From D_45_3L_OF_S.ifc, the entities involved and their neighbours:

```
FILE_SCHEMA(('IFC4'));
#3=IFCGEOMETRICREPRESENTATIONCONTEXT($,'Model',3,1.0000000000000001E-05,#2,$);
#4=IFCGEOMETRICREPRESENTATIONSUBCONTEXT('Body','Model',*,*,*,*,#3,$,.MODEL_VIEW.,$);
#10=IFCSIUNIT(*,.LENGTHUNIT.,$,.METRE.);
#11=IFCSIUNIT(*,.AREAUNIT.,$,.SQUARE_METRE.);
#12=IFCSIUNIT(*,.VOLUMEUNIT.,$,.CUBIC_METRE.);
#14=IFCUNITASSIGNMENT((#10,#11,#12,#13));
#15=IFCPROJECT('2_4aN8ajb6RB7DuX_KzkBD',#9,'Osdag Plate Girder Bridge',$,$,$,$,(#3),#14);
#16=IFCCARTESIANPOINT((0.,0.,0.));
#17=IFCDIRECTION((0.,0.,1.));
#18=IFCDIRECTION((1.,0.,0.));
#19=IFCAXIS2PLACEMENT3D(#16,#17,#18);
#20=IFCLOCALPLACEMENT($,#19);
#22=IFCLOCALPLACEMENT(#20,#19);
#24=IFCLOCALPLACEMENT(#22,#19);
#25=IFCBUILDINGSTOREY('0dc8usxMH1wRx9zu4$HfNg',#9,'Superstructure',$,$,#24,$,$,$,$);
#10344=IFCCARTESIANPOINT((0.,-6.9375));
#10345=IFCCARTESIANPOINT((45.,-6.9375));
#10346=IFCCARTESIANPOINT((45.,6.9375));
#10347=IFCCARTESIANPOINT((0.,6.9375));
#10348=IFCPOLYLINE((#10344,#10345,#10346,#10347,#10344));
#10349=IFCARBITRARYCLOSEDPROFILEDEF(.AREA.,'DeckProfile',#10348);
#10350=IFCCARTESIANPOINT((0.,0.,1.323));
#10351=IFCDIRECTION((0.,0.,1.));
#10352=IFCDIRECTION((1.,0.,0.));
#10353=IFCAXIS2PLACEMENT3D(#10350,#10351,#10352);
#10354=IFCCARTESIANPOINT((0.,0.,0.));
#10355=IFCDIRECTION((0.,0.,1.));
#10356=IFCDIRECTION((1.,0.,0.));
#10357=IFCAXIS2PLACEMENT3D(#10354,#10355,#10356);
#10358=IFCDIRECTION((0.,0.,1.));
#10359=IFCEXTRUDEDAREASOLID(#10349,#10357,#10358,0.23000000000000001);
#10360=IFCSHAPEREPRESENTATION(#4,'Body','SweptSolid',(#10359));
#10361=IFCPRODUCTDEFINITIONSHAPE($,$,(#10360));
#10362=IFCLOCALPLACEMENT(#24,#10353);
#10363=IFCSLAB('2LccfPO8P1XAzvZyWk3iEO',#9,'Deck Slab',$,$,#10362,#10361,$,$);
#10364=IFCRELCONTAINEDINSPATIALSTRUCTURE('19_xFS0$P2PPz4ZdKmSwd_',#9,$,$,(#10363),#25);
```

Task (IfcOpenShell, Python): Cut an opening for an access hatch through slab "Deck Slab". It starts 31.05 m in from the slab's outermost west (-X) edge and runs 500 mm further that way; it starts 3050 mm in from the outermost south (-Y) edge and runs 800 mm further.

```python
import numpy as np
import ifcopenshell
import ifcopenshell.api.feature
import ifcopenshell.api.geometry
import ifcopenshell.api.root
import ifcopenshell.geom
import ifcopenshell.util.placement
import ifcopenshell.util.representation
import ifcopenshell.util.shape
import ifcopenshell.util.unit

model = ifcopenshell.open("D_45_3L_OF_S.ifc")
unit_scale = ifcopenshell.util.unit.calculate_unit_scale(model)
settings = ifcopenshell.geom.settings()


def volume(element):
    """Net volume in cubic metres, openings subtracted."""
    shape = ifcopenshell.geom.create_shape(settings, element)
    return ifcopenshell.util.shape.get_volume(shape.geometry)


slab = model.by_id(10363)
before = volume(slab)

# Extent in the slab's own axes, in metres. The edges named are its -X and -Y sides.
slab_shape = ifcopenshell.geom.create_shape(settings, slab)
vertices = ifcopenshell.util.shape.get_vertices(slab_shape.geometry)
x_min, y_min, bottom = vertices.min(axis=0)
top = vertices[:, 2].max()

opening = ifcopenshell.api.root.create_entity(model, ifc_class="IfcOpeningElement", name="Access hatch opening", predefined_type="OPENING")
context = ifcopenshell.util.representation.get_context(model, "Model", "Body", "MODEL_VIEW")
width, depth = 0.5, 0.8
outline = [(0.0, 0.0), (width, 0.0), (width, depth), (0.0, depth), (0.0, 0.0)]
# Overshoot both faces by 50 mm so the cut is clean.
shape = ifcopenshell.api.geometry.add_slab_representation(
    model, context=context, depth=top - bottom + 0.1, polyline=outline
)
ifcopenshell.api.geometry.assign_representation(model, product=opening, representation=shape)

matrix = ifcopenshell.util.placement.get_local_placement(slab.ObjectPlacement)
matrix[:, 3] = matrix @ np.append(np.array([x_min + 31.05, y_min + 3.05, bottom - 0.05]) / unit_scale, 1.0)
ifcopenshell.api.geometry.edit_object_placement(model, product=opening, matrix=matrix, is_si=False)
ifcopenshell.api.feature.add_feature(model, feature=opening, element=slab)

after = volume(slab)

print(f"slab volume {before:.3f} -> {after:.3f} m3")

model.write("D_45_3L_OF_S_v2.ifc")
```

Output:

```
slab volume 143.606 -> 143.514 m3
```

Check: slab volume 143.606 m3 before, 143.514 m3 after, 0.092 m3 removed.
